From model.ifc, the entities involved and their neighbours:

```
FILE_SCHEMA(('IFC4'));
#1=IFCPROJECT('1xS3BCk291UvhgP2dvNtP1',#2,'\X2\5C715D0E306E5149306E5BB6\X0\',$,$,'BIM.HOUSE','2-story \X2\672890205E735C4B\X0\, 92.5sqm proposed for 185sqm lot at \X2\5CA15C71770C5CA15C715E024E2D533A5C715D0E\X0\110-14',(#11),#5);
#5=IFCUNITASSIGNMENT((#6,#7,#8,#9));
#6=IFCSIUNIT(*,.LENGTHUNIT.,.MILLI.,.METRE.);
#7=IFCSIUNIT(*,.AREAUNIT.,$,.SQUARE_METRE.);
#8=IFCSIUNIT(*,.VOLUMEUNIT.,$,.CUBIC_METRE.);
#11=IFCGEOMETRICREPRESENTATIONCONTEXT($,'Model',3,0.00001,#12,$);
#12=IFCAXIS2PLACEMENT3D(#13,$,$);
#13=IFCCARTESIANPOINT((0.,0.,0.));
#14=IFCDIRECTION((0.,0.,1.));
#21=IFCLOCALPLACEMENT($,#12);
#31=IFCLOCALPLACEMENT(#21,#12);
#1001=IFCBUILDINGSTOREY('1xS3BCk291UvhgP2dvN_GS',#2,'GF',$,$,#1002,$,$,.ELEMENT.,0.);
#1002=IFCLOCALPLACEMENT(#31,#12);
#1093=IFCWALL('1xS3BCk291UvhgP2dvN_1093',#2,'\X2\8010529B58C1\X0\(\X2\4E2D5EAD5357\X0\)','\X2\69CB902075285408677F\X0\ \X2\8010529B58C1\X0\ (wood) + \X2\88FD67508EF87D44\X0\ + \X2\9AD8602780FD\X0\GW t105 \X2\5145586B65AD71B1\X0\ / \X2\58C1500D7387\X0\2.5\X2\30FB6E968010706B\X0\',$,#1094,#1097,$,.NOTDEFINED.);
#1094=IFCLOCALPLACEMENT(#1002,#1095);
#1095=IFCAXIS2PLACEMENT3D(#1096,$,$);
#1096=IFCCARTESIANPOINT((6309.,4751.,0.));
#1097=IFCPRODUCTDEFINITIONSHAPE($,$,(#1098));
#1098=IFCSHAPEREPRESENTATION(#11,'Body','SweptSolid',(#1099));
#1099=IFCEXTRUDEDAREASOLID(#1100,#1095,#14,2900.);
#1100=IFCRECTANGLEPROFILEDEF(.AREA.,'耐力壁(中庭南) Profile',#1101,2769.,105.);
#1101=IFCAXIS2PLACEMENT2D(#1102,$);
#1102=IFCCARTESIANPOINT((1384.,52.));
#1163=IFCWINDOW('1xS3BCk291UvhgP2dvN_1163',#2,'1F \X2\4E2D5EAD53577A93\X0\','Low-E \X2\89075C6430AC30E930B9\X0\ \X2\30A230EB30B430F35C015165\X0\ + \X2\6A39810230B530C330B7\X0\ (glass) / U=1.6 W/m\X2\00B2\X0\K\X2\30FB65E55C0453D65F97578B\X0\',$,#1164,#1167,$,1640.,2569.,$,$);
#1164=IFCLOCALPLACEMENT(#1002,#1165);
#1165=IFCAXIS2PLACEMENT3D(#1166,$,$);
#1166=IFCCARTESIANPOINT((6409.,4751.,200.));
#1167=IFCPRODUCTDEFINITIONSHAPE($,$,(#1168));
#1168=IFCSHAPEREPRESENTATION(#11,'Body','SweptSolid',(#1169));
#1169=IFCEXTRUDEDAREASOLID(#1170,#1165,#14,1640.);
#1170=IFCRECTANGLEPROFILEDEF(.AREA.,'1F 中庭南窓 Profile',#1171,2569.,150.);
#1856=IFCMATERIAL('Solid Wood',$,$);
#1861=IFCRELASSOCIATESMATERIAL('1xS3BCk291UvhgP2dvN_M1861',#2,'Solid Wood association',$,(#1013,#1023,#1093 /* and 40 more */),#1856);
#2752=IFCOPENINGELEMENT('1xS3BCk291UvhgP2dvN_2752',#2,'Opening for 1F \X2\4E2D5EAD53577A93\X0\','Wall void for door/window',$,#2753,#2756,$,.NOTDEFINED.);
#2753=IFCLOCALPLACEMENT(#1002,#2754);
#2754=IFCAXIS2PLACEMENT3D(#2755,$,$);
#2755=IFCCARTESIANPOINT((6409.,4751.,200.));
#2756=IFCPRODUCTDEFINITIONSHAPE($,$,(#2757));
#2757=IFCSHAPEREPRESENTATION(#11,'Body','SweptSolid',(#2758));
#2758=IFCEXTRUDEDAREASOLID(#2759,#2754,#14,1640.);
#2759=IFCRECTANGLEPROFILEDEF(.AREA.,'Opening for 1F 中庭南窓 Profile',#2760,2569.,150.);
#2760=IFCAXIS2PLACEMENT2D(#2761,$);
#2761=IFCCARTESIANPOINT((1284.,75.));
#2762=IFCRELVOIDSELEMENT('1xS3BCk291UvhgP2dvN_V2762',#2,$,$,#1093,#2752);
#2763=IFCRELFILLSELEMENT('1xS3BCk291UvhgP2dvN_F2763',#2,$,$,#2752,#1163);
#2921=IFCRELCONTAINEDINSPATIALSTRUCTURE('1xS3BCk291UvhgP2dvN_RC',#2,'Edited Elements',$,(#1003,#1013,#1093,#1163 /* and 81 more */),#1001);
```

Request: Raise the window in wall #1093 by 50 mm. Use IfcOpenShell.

```python
import numpy as np
import ifcopenshell
import ifcopenshell.api.geometry
import ifcopenshell.util.placement
import ifcopenshell.util.unit

model = ifcopenshell.open("model.ifc")
unit_scale = ifcopenshell.util.unit.calculate_unit_scale(model)

window = model.by_guid("1xS3BCk291UvhgP2dvN_1163")
opening = window.FillsVoids[0].RelatingOpeningElement
dz = 0.05 / unit_scale

shift = np.array([0.0, 0.0, dz])
# The window is not placed relative to its opening, so move both.
for product in (opening, window):
    matrix = ifcopenshell.util.placement.get_local_placement(product.ObjectPlacement)
    matrix[:3, 3] += shift
    ifcopenshell.api.geometry.edit_object_placement(model, product=product, matrix=matrix, is_si=False)

print(f"moved by {dz * unit_scale:+.3f} m")

model.write("model_edited.ifc")
```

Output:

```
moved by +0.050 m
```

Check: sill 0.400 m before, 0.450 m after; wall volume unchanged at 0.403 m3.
